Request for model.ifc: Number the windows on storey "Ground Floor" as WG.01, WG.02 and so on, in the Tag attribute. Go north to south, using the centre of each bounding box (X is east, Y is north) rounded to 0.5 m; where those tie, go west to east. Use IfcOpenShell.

First a look at what the model holds.

```python
import ifcopenshell
import ifcopenshell.util.element
import ifcopenshell.util.placement

model = ifcopenshell.open("model.ifc")
print(model.schema)
storey = next(s for s in model.by_type("IfcBuildingStorey") if s.Name == "Ground Floor")
windows = [e for e in ifcopenshell.util.element.get_decomposition(storey) if e.is_a("IfcWindow")]
for e in sorted(windows, key=lambda e: e.id()):
    origin = ifcopenshell.util.placement.get_local_placement(e.ObjectPlacement)[:3, 3]
    print(e.id(), e.Tag, e.Name, origin.round(2) + 0.0, sep=" | ")
```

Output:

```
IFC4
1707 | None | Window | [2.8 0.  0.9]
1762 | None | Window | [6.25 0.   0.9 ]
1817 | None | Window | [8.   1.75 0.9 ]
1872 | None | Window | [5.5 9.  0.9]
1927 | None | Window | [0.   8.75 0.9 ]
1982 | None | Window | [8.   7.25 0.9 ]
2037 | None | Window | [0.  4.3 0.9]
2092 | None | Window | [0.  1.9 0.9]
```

```python
import ifcopenshell
import ifcopenshell.geom
import ifcopenshell.util.element
import ifcopenshell.util.shape

model = ifcopenshell.open("model.ifc")
settings = ifcopenshell.geom.settings()
settings.set("use-world-coords", True)


def centre(element):
    shape = ifcopenshell.geom.create_shape(settings, element)
    return ifcopenshell.util.shape.get_bbox_centroid(shape.geometry)


storey = next(s for s in model.by_type("IfcBuildingStorey") if s.Name == "Ground Floor")
windows = [e for e in ifcopenshell.util.element.get_decomposition(storey) if e.is_a("IfcWindow")]

# Insertion points can sit at a corner or the storey origin, so sort by the geometry (in metres).
centres = {e: centre(e) for e in windows}
windows.sort(key=lambda e: (-round(centres[e][1] / 0.5), centres[e][0]))

for i, e in enumerate(windows, start=1):
    number = f"WG.{i:02d}"
    e.Tag = number
    print(e.id(), number)

model.write("model_edited.ifc")
```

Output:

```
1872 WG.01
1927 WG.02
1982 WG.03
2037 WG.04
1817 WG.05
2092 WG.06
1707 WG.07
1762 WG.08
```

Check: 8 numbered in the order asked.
